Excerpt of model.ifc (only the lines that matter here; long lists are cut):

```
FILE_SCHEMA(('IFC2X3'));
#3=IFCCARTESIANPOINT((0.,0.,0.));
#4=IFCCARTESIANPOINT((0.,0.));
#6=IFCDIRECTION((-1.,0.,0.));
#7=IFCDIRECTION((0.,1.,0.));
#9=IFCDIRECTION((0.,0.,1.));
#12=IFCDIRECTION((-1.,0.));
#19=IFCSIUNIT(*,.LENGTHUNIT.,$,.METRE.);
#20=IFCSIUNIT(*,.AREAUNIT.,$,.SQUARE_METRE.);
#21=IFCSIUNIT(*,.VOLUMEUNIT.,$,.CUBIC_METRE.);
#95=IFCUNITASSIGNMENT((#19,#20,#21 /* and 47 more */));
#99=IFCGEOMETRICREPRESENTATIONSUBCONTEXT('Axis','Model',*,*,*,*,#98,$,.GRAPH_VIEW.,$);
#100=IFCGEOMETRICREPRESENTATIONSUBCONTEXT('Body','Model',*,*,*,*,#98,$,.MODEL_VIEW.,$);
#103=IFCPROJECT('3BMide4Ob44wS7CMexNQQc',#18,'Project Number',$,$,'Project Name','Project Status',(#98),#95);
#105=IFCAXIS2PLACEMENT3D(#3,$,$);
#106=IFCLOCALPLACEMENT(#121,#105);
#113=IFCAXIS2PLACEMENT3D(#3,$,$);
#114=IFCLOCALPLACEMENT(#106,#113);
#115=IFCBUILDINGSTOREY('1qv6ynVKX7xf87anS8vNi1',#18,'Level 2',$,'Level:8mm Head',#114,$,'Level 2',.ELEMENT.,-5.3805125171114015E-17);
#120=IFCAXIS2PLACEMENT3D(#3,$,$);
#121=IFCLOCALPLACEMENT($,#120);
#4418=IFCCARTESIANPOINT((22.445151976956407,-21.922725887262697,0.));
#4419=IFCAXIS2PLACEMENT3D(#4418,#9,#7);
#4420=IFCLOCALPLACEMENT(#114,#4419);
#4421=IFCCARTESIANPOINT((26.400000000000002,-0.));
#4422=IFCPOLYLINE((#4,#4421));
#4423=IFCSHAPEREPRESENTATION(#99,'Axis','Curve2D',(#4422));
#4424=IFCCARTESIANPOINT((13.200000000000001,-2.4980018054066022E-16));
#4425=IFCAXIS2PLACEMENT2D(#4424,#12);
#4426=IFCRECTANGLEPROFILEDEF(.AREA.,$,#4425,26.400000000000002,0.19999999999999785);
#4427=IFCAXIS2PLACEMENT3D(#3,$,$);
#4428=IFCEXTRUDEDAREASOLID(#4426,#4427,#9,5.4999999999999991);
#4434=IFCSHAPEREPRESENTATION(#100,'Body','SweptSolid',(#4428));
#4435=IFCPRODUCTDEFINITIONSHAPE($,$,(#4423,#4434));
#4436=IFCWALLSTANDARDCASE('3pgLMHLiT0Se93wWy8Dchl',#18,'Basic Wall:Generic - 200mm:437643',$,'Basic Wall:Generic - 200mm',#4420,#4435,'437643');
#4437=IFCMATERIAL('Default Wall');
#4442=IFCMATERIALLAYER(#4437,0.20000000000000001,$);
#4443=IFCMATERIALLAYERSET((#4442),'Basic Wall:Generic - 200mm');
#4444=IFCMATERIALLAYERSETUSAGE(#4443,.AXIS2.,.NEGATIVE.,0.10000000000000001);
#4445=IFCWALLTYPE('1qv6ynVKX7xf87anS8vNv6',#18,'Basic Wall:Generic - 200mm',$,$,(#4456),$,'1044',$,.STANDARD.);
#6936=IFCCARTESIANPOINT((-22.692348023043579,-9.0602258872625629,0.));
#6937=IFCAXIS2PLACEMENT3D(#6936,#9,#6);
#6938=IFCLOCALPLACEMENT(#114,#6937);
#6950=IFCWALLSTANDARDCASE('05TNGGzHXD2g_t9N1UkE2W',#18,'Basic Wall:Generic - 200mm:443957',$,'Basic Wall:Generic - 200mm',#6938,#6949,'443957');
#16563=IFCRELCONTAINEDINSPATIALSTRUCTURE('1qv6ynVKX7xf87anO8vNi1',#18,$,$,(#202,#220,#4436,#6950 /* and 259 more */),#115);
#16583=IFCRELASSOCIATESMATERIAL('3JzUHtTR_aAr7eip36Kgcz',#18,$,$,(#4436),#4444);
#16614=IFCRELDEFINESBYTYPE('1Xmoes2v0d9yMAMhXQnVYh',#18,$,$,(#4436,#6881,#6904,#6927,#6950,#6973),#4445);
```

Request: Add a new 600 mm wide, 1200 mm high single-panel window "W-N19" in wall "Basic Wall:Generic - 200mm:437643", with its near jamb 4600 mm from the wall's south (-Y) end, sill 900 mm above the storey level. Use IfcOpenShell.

```python
import numpy as np
import ifcopenshell
import ifcopenshell.api.feature
import ifcopenshell.api.geometry
import ifcopenshell.api.root
import ifcopenshell.api.spatial
import ifcopenshell.api.type
import ifcopenshell.geom
import ifcopenshell.util.element
import ifcopenshell.util.placement
import ifcopenshell.util.representation
import ifcopenshell.util.shape
import ifcopenshell.util.unit

model = ifcopenshell.open("model.ifc")
unit_scale = ifcopenshell.util.unit.calculate_unit_scale(model)
settings = ifcopenshell.geom.settings()


def volume(element):
    """Net volume in cubic metres, openings subtracted."""
    shape = ifcopenshell.geom.create_shape(settings, element)
    return ifcopenshell.util.shape.get_volume(shape.geometry)


wall = model.by_id(4436)
storey = ifcopenshell.util.element.get_container(wall, ifc_class="IfcBuildingStorey")
context = ifcopenshell.util.representation.get_context(model, "Model", "Body", "MODEL_VIEW")
before = volume(wall)

width, height, from_end, sill = 0.6, 1.2, 4.6, 0.9  # metres

# The wall runs along its own X axis, and the end named is its -X end.
wall_shape = ifcopenshell.geom.create_shape(settings, wall)
x, y, z = ifcopenshell.util.shape.get_vertices(wall_shape.geometry).T
start = x.min() + from_end
face, thickness = float(y.min()), float(y.max() - y.min())
wall_matrix = ifcopenshell.util.placement.get_local_placement(wall.ObjectPlacement)
level = ifcopenshell.util.placement.get_local_placement(storey.ObjectPlacement)[2, 3]


def in_wall(x, y):
    """Placement at x, y metres in the wall's axes, at sill height."""
    matrix = wall_matrix.copy()
    matrix[:, 3] = wall_matrix @ np.array([x / unit_scale, y / unit_scale, 0.0, 1.0])
    matrix[2, 3] = level + sill / unit_scale
    return matrix


# Opening: a box that overshoots both wall faces by 50 mm.
opening = ifcopenshell.api.root.create_entity(model, ifc_class="IfcOpeningElement")
box = ifcopenshell.api.geometry.add_wall_representation(
    model, context=context, length=width, height=height, thickness=thickness + 0.1
)
ifcopenshell.api.geometry.assign_representation(model, product=opening, representation=box)
ifcopenshell.api.geometry.edit_object_placement(model, product=opening, matrix=in_wall(start, face - 0.05), is_si=False)
ifcopenshell.api.feature.add_feature(model, feature=opening, element=wall)

window = ifcopenshell.api.root.create_entity(model, ifc_class="IfcWindow", name="W-N19")
window.OverallWidth, window.OverallHeight = width / unit_scale, height / unit_scale
body = ifcopenshell.api.geometry.add_window_representation(
    model,
    context=context,
    overall_width=window.OverallWidth,
    overall_height=window.OverallHeight,
    partition_type="SINGLE_PANEL",
)
ifcopenshell.api.geometry.assign_representation(model, product=window, representation=body)
ifcopenshell.api.spatial.assign_container(model, products=[window], relating_structure=storey)
fills = ifcopenshell.api.feature.add_filling(model, opening=opening, element=window)
fills.OwnerHistory = window.OwnerHistory  # required in IFC2X3

# IFC2X3 keeps the operation on the window style.
style = ifcopenshell.api.root.create_entity(model, ifc_class="IfcWindowStyle", name="W-N19")
style.OperationType, style.ConstructionType = "SINGLE_PANEL", "NOTDEFINED"
style.ParameterTakesPrecedence = style.Sizeable = False
ifcopenshell.api.type.assign_type(model, related_objects=[window], relating_type=style)

# Centre the window in the wall's thickness.
ifcopenshell.api.geometry.edit_object_placement(model, product=window, matrix=in_wall(start, face), is_si=False)
window_shape = ifcopenshell.geom.create_shape(settings, window)
depth = ifcopenshell.util.shape.get_vertices(window_shape.geometry)[:, 1]
offset = face + thickness / 2 - (depth.min() + depth.max()) / 2
ifcopenshell.api.geometry.edit_object_placement(model, product=window, matrix=in_wall(start, offset), is_si=False)

after = volume(wall)

print(f"wall volume {before:.3f} -> {after:.3f} m3")

model.write("model-out.ifc")
```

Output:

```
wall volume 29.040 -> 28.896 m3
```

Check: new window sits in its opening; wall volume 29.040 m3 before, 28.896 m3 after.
